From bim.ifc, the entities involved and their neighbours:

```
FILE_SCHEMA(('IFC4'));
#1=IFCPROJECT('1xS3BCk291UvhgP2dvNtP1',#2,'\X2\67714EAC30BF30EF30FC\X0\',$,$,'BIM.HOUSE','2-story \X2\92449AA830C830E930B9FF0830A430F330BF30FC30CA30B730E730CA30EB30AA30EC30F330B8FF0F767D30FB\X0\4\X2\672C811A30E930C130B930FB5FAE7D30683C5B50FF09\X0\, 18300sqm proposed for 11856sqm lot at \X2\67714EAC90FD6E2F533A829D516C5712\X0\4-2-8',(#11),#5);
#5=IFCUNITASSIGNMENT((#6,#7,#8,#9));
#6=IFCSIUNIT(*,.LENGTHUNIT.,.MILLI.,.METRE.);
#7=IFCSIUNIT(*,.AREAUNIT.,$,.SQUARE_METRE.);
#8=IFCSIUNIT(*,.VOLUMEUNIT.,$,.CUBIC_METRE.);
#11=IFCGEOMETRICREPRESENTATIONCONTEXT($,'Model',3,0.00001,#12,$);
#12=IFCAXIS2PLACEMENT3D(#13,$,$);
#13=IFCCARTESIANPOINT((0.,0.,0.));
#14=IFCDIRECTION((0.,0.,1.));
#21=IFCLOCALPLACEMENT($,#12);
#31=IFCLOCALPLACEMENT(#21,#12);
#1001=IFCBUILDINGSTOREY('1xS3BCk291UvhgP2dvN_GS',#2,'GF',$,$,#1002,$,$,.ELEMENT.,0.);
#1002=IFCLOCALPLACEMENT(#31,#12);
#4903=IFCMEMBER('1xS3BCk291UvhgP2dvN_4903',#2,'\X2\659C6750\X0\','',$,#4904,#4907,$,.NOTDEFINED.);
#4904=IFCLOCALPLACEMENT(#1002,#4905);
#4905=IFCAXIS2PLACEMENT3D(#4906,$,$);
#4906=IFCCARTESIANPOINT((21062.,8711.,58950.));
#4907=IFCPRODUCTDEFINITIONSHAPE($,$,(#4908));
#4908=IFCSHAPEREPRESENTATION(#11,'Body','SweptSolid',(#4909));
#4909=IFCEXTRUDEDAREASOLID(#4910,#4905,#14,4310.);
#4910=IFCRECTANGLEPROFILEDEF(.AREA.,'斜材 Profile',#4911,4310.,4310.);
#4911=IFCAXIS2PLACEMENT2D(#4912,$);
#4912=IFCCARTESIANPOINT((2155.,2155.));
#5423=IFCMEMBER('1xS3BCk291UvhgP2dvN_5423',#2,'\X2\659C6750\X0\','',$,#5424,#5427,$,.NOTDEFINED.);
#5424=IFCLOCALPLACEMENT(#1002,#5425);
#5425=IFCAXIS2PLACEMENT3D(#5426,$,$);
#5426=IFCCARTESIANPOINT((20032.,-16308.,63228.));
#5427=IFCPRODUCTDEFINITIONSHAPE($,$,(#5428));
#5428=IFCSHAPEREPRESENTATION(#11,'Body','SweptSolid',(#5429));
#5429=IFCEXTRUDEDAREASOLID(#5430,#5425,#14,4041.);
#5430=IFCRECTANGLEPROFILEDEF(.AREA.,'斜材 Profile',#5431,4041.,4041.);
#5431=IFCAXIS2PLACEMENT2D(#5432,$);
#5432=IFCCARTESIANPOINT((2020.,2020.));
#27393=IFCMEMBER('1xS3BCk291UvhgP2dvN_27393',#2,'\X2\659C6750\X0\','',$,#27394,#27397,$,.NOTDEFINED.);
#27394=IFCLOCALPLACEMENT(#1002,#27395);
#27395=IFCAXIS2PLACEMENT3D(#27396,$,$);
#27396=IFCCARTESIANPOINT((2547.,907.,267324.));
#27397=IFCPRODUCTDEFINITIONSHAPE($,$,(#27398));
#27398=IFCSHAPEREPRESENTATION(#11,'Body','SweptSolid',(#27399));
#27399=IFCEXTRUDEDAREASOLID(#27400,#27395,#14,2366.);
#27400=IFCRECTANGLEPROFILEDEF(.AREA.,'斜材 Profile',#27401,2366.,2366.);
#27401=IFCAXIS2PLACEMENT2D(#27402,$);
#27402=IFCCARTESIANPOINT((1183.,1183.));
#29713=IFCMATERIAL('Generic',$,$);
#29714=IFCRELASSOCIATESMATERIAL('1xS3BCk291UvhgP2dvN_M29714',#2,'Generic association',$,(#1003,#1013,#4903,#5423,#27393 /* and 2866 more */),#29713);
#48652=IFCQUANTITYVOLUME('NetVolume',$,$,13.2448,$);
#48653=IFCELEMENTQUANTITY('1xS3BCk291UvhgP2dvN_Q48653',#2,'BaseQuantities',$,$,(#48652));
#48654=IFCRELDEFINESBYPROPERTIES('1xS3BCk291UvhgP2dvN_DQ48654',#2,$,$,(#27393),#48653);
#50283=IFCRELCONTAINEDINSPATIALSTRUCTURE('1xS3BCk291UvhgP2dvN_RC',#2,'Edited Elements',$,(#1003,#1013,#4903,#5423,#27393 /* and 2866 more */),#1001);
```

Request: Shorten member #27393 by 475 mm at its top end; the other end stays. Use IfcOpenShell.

```python
import ifcopenshell
import ifcopenshell.api.pset
import ifcopenshell.util.element
import ifcopenshell.util.unit

model = ifcopenshell.open("bim.ifc")
unit_scale = ifcopenshell.util.unit.calculate_unit_scale(model)

member = model.by_guid("1xS3BCk291UvhgP2dvN_27393")
change = -0.475 / unit_scale

# The extrusion runs towards the end named, so only its depth changes.
body = next(r for r in member.Representation.Representations if r.RepresentationIdentifier == "Body")
solid = body.Items[0]
old_length = solid.Depth
solid.Depth += change

# Update the stored length and volume.
qto = model.by_id(ifcopenshell.util.element.get_pset(member, "BaseQuantities", should_inherit=False)["id"])
ifcopenshell.api.pset.edit_qto(model, qto=qto, properties={
    "NetVolume": ifcopenshell.util.element.get_pset(member, "BaseQuantities", "NetVolume") * solid.Depth / old_length,
})

print(f"length {old_length:g} -> {solid.Depth:g}")

model.write("bim_updated.ifc")
```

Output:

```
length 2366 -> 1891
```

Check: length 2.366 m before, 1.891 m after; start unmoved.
